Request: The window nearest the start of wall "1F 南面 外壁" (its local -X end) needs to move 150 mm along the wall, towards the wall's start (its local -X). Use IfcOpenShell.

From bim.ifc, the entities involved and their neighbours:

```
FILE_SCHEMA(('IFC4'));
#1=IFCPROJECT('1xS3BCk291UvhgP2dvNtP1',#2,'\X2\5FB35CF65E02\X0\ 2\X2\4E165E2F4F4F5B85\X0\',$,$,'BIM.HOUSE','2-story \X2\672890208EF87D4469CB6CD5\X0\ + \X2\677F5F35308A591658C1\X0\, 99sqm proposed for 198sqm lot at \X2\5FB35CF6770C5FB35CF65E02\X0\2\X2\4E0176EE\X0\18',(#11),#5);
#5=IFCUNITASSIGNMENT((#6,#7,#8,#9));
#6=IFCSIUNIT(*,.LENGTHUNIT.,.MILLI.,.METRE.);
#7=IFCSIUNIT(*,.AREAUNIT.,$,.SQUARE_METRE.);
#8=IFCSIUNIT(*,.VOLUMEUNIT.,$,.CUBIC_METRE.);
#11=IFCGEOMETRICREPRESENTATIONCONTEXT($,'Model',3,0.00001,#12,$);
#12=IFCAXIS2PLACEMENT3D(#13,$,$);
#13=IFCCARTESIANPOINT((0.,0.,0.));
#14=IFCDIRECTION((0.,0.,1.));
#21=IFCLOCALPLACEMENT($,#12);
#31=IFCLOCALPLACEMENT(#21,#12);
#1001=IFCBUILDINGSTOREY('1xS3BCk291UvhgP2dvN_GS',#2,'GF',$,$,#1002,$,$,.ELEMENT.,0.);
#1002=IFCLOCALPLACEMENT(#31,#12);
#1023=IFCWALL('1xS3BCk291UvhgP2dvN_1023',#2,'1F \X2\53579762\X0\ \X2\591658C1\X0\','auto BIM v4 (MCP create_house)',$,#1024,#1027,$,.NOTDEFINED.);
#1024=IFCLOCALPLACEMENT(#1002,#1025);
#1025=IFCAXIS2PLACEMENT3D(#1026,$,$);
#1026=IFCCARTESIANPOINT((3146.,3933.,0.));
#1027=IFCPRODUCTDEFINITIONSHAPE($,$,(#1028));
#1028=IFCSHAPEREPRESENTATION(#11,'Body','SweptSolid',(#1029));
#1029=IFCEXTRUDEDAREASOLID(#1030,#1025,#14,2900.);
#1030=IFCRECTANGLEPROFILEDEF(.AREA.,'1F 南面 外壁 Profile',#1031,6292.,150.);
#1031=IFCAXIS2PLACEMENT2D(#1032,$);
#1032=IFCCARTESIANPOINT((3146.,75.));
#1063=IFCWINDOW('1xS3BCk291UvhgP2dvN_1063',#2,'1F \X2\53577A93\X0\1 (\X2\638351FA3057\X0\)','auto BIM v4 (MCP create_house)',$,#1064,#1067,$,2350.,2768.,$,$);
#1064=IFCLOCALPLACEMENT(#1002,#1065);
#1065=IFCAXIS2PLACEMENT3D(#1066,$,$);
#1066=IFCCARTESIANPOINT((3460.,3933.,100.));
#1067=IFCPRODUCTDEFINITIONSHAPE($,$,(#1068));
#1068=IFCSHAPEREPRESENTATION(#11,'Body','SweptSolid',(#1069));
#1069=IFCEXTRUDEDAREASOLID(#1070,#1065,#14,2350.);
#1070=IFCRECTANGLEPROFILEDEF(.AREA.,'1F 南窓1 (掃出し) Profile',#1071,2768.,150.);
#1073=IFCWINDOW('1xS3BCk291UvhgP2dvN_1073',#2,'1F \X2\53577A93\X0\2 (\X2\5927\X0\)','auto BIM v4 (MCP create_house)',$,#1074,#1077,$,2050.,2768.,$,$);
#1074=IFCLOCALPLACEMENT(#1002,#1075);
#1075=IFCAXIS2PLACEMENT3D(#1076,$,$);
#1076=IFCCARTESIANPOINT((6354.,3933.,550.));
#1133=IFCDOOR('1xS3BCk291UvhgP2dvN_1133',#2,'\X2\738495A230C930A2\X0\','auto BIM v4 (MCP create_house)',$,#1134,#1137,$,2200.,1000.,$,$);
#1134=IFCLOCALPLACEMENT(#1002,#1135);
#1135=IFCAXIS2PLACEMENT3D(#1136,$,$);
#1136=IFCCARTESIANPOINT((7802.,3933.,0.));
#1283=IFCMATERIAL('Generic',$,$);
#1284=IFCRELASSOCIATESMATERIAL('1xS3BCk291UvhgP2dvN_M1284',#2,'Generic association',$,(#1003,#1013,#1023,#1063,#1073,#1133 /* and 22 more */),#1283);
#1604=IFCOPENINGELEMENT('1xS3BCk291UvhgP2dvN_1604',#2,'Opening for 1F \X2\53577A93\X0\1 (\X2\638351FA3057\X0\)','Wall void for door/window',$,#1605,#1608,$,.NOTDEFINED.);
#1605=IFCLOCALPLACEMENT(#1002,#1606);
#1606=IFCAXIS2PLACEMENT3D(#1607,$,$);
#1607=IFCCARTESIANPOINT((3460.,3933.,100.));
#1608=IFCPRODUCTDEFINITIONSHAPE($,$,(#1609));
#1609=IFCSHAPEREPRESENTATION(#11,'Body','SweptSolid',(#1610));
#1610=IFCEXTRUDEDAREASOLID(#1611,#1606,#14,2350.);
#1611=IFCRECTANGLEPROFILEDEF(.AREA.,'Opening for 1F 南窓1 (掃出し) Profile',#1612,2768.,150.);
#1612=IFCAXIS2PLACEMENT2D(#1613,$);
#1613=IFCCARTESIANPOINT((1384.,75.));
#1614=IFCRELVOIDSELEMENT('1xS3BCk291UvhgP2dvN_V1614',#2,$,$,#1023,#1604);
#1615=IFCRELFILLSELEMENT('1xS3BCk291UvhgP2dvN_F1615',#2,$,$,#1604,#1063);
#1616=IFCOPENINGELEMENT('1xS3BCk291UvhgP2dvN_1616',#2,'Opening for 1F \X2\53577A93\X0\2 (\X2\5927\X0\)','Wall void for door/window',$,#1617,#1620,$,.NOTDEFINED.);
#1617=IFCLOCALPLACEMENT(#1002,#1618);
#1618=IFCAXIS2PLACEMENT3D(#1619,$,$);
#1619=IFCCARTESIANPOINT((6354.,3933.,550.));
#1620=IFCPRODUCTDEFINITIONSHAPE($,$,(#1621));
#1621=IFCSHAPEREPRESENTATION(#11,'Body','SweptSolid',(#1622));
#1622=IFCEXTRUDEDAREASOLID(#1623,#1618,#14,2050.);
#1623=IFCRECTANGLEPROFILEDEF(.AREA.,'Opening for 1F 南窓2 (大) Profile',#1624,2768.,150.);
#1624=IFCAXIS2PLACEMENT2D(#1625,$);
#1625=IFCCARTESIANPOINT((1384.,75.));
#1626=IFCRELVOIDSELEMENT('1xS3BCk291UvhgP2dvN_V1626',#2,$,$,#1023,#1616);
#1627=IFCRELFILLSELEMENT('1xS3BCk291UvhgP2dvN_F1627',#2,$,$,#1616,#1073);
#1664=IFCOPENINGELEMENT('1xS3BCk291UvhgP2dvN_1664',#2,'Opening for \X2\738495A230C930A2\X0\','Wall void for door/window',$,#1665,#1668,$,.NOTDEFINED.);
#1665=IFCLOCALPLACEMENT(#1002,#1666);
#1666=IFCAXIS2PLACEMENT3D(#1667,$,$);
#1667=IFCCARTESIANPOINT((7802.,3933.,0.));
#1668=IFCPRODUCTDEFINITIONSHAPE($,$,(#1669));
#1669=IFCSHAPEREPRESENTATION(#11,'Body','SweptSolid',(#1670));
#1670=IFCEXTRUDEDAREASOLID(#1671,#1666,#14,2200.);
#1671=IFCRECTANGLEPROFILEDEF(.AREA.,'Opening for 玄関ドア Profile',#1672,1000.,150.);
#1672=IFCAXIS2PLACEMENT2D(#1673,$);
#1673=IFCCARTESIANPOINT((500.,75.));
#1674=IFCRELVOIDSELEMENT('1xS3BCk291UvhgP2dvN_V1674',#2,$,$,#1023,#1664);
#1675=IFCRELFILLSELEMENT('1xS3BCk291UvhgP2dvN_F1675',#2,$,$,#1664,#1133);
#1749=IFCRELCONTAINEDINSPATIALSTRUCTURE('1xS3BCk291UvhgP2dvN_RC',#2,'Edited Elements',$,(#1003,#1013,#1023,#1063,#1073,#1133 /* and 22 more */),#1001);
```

```python
import ifcopenshell
import ifcopenshell.api.geometry
import ifcopenshell.util.placement
import ifcopenshell.util.unit

model = ifcopenshell.open("bim.ifc")
unit_scale = ifcopenshell.util.unit.calculate_unit_scale(model)

window = model.by_id(1063)
opening = window.FillsVoids[0].RelatingOpeningElement
wall = opening.VoidsElements[0].RelatingBuildingElement

wall_matrix = ifcopenshell.util.placement.get_local_placement(wall.ObjectPlacement)
shift = wall_matrix[:3, 0] * -0.15 / unit_scale
before = ifcopenshell.util.placement.get_local_placement(window.ObjectPlacement)[:3, 3].copy()

# The window is not placed relative to its opening, so move both.
for product in (opening, window):
    matrix = ifcopenshell.util.placement.get_local_placement(product.ObjectPlacement)
    matrix[:3, 3] += shift
    ifcopenshell.api.geometry.edit_object_placement(model, product=product, matrix=matrix, is_si=False)

after = ifcopenshell.util.placement.get_local_placement(window.ObjectPlacement)[:3, 3]
print("window moved by", (after - before).round(3) + 0.0)

model.write("bim_rev.ifc")
```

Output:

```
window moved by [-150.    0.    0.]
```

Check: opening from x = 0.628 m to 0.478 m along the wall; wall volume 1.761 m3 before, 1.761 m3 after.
